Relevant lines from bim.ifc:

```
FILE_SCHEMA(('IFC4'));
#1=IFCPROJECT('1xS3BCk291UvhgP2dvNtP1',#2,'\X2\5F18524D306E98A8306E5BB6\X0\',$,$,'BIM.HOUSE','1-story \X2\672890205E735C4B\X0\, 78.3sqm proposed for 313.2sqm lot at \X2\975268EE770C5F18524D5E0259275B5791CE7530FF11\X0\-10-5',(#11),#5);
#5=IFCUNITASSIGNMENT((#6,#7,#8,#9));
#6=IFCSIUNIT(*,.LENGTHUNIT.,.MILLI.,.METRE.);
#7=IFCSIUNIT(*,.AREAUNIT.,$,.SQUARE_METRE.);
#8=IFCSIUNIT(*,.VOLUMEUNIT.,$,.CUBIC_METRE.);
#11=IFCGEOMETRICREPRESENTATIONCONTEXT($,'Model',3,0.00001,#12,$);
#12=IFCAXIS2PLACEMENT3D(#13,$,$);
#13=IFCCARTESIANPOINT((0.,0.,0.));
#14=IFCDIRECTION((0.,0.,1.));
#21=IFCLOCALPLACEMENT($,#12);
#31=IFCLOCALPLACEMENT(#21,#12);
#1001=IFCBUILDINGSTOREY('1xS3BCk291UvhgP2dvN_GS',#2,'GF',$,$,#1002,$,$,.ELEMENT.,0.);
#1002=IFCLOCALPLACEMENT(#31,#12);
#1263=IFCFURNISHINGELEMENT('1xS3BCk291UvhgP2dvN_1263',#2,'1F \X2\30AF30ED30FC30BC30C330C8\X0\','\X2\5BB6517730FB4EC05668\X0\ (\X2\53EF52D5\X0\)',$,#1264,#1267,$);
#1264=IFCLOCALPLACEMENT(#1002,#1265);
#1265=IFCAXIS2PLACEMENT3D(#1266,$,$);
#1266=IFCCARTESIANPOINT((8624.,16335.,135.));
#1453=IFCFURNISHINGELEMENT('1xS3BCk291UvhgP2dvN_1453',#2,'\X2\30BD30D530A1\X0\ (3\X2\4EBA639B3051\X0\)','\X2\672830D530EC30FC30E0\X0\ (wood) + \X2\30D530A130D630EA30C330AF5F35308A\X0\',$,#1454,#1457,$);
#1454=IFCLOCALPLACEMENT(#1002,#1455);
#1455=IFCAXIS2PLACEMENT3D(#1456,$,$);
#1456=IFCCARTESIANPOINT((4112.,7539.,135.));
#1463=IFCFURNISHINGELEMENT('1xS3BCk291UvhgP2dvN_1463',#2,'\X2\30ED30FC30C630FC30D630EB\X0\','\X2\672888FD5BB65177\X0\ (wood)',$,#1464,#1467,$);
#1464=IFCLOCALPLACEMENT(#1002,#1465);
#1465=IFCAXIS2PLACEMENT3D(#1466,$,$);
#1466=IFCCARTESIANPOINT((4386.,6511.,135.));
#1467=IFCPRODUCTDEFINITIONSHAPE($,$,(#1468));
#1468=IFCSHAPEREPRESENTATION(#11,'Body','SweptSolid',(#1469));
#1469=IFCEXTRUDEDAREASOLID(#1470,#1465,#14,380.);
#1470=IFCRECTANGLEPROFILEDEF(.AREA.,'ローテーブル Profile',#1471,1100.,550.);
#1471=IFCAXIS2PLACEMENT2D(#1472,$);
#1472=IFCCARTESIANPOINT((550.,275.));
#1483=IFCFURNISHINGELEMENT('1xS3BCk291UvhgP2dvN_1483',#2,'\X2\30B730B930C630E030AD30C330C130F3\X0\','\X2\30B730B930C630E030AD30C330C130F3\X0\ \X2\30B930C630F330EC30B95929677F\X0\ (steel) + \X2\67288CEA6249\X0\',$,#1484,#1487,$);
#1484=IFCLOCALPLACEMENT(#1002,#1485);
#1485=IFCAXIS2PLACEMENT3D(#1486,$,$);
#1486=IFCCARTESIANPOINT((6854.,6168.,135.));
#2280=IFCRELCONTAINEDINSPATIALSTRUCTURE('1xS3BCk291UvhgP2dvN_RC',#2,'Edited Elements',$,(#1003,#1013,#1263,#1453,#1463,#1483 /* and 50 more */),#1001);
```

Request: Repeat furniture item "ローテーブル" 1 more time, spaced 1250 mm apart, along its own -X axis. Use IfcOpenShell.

```python
import ifcopenshell
import ifcopenshell.api.geometry
import ifcopenshell.api.root
import ifcopenshell.util.element
import ifcopenshell.util.placement

model = ifcopenshell.open("bim.ifc")


def reuse_history(source, copy):
    """copy_class also copies each property set's owner history, people and application; keep the originals."""
    for rel in copy.IsDefinedBy:
        if rel.is_a("IfcRelDefinesByProperties") and (history := rel.RelatingPropertyDefinition.OwnerHistory):
            rel.RelatingPropertyDefinition.OwnerHistory = source.OwnerHistory
            ifcopenshell.util.element.remove_deep2(model, history)


source = model.by_guid("1xS3BCk291UvhgP2dvN_1463")
base = ifcopenshell.util.placement.get_local_placement(source.ObjectPlacement)
step = -base[:3, 0] * 1250.0

for i in range(1, 2):
    copy = ifcopenshell.api.root.copy_class(model, product=source)
    copy.Representation = ifcopenshell.util.element.copy_deep(
        model, source.Representation, exclude=["IfcGeometricRepresentationContext", "IfcRepresentationMap"]
    )
    reuse_history(source, copy)
    matrix = base.copy()
    matrix[:3, 3] += i * step
    print("added at", matrix[:3, 3].round(3) + 0.0)
    ifcopenshell.api.geometry.edit_object_placement(model, product=copy, matrix=matrix, is_si=False)

model.write("bim_v2.ifc")
```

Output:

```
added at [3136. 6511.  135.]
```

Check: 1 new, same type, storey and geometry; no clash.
